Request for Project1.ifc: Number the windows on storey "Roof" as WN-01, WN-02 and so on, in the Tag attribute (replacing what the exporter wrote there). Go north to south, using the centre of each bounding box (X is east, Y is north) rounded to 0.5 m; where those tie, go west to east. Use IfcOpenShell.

First a look at what the model holds.

```python
import ifcopenshell
import ifcopenshell.util.element
import ifcopenshell.util.placement

model = ifcopenshell.open("Project1.ifc")
print(model.schema)
storey = next(s for s in model.by_type("IfcBuildingStorey") if s.Name == "Roof")
windows = [e for e in ifcopenshell.util.element.get_decomposition(storey) if e.is_a("IfcWindow")]
for e in sorted(windows, key=lambda e: e.id()):
    origin = ifcopenshell.util.placement.get_local_placement(e.ObjectPlacement)[:3, 3]
    print(e.id(), e.Tag, e.Name, origin.round(2) + 0.0, sep=" | ")
```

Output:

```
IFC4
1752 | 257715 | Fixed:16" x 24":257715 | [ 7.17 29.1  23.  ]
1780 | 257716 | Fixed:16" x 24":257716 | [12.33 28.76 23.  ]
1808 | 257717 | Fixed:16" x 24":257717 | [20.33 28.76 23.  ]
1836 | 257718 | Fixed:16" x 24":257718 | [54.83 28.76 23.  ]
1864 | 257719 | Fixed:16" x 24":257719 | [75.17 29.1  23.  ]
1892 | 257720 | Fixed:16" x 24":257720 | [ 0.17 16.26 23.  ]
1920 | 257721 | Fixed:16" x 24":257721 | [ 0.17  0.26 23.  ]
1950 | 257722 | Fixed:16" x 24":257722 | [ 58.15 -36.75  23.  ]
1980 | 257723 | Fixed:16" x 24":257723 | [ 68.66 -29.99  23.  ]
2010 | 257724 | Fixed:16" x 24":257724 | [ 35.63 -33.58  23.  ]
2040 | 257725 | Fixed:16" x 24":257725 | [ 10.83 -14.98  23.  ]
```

```python
import ifcopenshell
import ifcopenshell.geom
import ifcopenshell.util.element
import ifcopenshell.util.shape

model = ifcopenshell.open("Project1.ifc")
settings = ifcopenshell.geom.settings()
settings.set("use-world-coords", True)


def centre(element):
    shape = ifcopenshell.geom.create_shape(settings, element)
    return ifcopenshell.util.shape.get_bbox_centroid(shape.geometry)


storey = next(s for s in model.by_type("IfcBuildingStorey") if s.Name == "Roof")
windows = [e for e in ifcopenshell.util.element.get_decomposition(storey) if e.is_a("IfcWindow")]

# Insertion points can sit at a corner or the storey origin, so sort by the geometry (in metres).
centres = {e: centre(e) for e in windows}
windows.sort(key=lambda e: (-round(centres[e][1] / 0.5), centres[e][0]))

for i, e in enumerate(windows, start=1):
    number = f"WN-{i:02d}"
    e.Tag = number
    print(e.id(), number)

model.write("Project1_updated.ifc")
```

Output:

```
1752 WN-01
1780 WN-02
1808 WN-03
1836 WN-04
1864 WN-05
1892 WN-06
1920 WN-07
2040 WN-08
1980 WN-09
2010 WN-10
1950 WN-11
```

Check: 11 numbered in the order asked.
